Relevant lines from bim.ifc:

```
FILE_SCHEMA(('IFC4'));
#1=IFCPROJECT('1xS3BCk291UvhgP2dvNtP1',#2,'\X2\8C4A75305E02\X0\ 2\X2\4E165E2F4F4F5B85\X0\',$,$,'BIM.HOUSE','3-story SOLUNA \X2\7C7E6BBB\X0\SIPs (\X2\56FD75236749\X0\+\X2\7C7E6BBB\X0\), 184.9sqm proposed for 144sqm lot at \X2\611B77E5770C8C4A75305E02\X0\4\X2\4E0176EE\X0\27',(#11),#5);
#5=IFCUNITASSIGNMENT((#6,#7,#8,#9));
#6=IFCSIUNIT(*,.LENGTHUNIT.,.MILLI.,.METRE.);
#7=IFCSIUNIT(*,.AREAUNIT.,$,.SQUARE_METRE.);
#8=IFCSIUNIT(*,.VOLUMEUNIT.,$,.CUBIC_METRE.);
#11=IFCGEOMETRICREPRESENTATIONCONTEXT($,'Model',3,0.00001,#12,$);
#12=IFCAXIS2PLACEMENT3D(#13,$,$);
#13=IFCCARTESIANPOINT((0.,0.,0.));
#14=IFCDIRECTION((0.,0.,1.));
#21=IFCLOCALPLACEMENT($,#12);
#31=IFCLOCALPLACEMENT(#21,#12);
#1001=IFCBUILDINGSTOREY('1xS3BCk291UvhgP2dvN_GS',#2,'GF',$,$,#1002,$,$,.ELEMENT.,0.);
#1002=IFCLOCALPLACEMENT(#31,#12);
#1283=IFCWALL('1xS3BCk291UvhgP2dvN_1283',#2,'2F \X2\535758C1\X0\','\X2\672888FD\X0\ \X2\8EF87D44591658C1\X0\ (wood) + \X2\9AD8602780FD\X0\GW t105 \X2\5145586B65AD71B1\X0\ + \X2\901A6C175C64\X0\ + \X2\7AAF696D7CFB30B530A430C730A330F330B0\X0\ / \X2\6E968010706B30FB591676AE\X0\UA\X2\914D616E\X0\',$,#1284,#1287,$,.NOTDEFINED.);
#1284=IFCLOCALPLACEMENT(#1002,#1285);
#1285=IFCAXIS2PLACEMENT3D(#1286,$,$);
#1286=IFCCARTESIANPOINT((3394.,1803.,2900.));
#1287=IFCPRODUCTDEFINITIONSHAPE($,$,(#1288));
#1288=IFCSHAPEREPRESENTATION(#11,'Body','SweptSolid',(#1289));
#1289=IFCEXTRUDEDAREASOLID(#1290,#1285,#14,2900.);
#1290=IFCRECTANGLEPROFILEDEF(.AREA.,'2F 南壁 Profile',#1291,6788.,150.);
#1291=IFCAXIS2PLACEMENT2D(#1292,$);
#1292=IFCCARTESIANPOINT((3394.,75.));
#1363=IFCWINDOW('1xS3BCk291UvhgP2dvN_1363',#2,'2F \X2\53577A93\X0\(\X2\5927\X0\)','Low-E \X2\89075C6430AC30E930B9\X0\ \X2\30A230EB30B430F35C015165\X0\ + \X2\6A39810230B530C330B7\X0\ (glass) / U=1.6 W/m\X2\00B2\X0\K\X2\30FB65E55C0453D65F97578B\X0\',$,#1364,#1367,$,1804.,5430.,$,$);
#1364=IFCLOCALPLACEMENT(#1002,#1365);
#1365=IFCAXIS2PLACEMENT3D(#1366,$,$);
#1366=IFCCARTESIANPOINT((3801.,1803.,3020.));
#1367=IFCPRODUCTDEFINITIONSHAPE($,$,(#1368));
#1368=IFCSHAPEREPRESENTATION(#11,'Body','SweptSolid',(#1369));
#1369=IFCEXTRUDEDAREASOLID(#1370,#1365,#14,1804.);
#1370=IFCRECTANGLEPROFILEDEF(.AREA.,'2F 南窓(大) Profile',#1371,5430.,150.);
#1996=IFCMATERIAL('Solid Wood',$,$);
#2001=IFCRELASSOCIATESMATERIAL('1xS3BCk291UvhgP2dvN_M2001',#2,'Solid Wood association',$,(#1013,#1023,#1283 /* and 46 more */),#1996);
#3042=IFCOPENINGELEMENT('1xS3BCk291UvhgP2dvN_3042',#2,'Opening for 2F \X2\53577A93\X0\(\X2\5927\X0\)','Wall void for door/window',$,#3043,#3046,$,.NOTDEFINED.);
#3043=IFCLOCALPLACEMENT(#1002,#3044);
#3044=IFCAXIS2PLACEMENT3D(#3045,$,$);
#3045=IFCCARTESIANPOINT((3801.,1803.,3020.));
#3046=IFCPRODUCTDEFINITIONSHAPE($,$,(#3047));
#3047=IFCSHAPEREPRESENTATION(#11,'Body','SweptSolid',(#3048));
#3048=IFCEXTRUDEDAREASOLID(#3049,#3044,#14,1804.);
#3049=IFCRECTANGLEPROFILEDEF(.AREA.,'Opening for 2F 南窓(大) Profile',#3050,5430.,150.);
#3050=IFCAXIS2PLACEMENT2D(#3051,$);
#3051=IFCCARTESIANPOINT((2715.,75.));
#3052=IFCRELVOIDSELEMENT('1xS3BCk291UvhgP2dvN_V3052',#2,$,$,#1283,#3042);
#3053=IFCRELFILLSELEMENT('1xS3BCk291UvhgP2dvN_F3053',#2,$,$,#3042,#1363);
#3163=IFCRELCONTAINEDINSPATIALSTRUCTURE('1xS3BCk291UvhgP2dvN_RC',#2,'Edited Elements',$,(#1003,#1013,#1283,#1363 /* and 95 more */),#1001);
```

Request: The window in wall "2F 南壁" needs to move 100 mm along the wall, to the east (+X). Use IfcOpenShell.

```python
import ifcopenshell
import ifcopenshell.api.geometry
import ifcopenshell.util.placement
import ifcopenshell.util.unit

model = ifcopenshell.open("bim.ifc")
unit_scale = ifcopenshell.util.unit.calculate_unit_scale(model)

window = model.by_guid("1xS3BCk291UvhgP2dvN_1363")
opening = window.FillsVoids[0].RelatingOpeningElement
wall = opening.VoidsElements[0].RelatingBuildingElement

wall_matrix = ifcopenshell.util.placement.get_local_placement(wall.ObjectPlacement)
shift = wall_matrix[:3, 0] * 0.1 / unit_scale
before = ifcopenshell.util.placement.get_local_placement(window.ObjectPlacement)[:3, 3].copy()

# The window is not placed relative to its opening, so move both.
for product in (opening, window):
    matrix = ifcopenshell.util.placement.get_local_placement(product.ObjectPlacement)
    matrix[:3, 3] += shift
    ifcopenshell.api.geometry.edit_object_placement(model, product=product, matrix=matrix, is_si=False)

after = ifcopenshell.util.placement.get_local_placement(window.ObjectPlacement)[:3, 3]
print("window moved by", (after - before).round(3) + 0.0)

model.write("bim_updated.ifc")
```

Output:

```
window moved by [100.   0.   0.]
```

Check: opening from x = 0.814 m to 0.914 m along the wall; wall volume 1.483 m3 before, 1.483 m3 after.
